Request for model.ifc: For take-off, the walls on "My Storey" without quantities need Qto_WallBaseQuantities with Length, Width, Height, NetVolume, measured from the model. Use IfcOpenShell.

First a look at what the model holds.

```python
import ifcopenshell
import ifcopenshell.util.element
import ifcopenshell.util.unit

model = ifcopenshell.open("model.ifc")
print(model.schema)
for unit_type in ("LENGTHUNIT", "AREAUNIT", "VOLUMEUNIT"):
    print(unit_type, ifcopenshell.util.unit.calculate_unit_scale(model, unit_type))
storey = next(s for s in model.by_type("IfcBuildingStorey") if s.Name == "My Storey")
walls = [e for e in ifcopenshell.util.element.get_decomposition(storey) if e.is_a("IfcWall")]
for e in sorted(walls, key=lambda e: e.id()):
    print(e.id(), e.is_a(), e.Name, list(ifcopenshell.util.element.get_psets(e, qtos_only=True)), sep=" | ")
```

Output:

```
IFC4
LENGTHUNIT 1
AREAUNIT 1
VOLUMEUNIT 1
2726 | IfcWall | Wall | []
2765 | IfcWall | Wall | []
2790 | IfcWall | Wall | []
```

```python
import ifcopenshell
import ifcopenshell.api.pset
import ifcopenshell.geom
import ifcopenshell.util.element
import ifcopenshell.util.shape
import ifcopenshell.util.unit

model = ifcopenshell.open("model.ifc")
unit_scale = ifcopenshell.util.unit.calculate_unit_scale(model)
volume_scale = ifcopenshell.util.unit.calculate_unit_scale(model, "VOLUMEUNIT")
settings = ifcopenshell.geom.settings()

storey = next(s for s in model.by_type("IfcBuildingStorey") if s.Name == "My Storey")
walls = [e for e in ifcopenshell.util.element.get_decomposition(storey) if e.is_a("IfcWall")]

for e in sorted(walls, key=lambda e: e.id()):
    if ifcopenshell.util.element.get_psets(e, qtos_only=True, should_inherit=False):
        continue
    # Geometry comes back in metres, in the element's own axes.
    shape = ifcopenshell.geom.create_shape(settings, e)
    values = {
        "Length": ifcopenshell.util.shape.get_x(shape.geometry) / unit_scale,
        "Width": ifcopenshell.util.shape.get_y(shape.geometry) / unit_scale,
        "Height": ifcopenshell.util.shape.get_z(shape.geometry) / unit_scale,
        "NetVolume": ifcopenshell.util.shape.get_volume(shape.geometry) / volume_scale,
    }
    qto = ifcopenshell.api.pset.add_qto(model, product=e, name="Qto_WallBaseQuantities")
    ifcopenshell.api.pset.edit_qto(model, qto=qto, properties=values)
    print(e.id(), {k: round(v, 3) for k, v in values.items()})

model.write("model_edited.ifc")
```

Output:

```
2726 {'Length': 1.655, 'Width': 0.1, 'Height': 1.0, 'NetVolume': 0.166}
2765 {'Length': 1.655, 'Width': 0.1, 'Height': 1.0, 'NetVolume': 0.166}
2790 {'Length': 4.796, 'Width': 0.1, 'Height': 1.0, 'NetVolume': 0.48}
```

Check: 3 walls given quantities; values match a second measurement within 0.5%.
